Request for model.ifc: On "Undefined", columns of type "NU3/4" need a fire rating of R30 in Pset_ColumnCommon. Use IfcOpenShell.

First a look at what the model holds.

```python
import ifcopenshell
import ifcopenshell.util.element

model = ifcopenshell.open("model.ifc")
print(model.schema)
storey = next(s for s in model.by_type("IfcBuildingStorey") if s.Name == "Undefined")
columns = [e for e in ifcopenshell.util.element.get_decomposition(storey) if e.is_a("IfcColumn")]
seen = {}
for e in columns:
    element_type = ifcopenshell.util.element.get_type(e)
    key = (element_type.Name if element_type != e and element_type else None, ifcopenshell.util.element.get_pset(e, "Pset_ColumnCommon", "FireRating"))
    seen[key] = seen.get(key, 0) + 1
for (name, value), count in sorted(seen.items(), key=str):
    print(count, "x", name, "|", value)
```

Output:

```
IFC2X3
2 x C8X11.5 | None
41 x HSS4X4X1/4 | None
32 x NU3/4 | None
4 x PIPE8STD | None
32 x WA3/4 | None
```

```python
import ifcopenshell
import ifcopenshell.api.pset
import ifcopenshell.util.element

model = ifcopenshell.open("model.ifc")

storey = next(s for s in model.by_type("IfcBuildingStorey") if s.Name == "Undefined")
columns = [e for e in ifcopenshell.util.element.get_decomposition(storey) if e.is_a("IfcColumn")]

count = 0
for e in columns:
    element_type = ifcopenshell.util.element.get_type(e)
    if element_type in (None, e) or element_type.Name != "NU3/4":
        continue
    found = ifcopenshell.util.element.get_pset(e, "Pset_ColumnCommon", should_inherit=False)
    if found:
        pset = model.by_id(found["id"])
        if len(ifcopenshell.util.element.get_elements_by_pset(pset)) > 1:
            pset = ifcopenshell.api.pset.unshare_pset(model, products=[e], pset=pset)[0]
    else:
        pset = ifcopenshell.api.pset.add_pset(model, product=e, name="Pset_ColumnCommon")
    ifcopenshell.api.pset.edit_pset(model, pset=pset, properties={"FireRating": "R30"})
    count += 1

print(count, "columns updated")

model.write("model_updated.ifc")
```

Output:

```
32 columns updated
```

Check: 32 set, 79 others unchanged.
